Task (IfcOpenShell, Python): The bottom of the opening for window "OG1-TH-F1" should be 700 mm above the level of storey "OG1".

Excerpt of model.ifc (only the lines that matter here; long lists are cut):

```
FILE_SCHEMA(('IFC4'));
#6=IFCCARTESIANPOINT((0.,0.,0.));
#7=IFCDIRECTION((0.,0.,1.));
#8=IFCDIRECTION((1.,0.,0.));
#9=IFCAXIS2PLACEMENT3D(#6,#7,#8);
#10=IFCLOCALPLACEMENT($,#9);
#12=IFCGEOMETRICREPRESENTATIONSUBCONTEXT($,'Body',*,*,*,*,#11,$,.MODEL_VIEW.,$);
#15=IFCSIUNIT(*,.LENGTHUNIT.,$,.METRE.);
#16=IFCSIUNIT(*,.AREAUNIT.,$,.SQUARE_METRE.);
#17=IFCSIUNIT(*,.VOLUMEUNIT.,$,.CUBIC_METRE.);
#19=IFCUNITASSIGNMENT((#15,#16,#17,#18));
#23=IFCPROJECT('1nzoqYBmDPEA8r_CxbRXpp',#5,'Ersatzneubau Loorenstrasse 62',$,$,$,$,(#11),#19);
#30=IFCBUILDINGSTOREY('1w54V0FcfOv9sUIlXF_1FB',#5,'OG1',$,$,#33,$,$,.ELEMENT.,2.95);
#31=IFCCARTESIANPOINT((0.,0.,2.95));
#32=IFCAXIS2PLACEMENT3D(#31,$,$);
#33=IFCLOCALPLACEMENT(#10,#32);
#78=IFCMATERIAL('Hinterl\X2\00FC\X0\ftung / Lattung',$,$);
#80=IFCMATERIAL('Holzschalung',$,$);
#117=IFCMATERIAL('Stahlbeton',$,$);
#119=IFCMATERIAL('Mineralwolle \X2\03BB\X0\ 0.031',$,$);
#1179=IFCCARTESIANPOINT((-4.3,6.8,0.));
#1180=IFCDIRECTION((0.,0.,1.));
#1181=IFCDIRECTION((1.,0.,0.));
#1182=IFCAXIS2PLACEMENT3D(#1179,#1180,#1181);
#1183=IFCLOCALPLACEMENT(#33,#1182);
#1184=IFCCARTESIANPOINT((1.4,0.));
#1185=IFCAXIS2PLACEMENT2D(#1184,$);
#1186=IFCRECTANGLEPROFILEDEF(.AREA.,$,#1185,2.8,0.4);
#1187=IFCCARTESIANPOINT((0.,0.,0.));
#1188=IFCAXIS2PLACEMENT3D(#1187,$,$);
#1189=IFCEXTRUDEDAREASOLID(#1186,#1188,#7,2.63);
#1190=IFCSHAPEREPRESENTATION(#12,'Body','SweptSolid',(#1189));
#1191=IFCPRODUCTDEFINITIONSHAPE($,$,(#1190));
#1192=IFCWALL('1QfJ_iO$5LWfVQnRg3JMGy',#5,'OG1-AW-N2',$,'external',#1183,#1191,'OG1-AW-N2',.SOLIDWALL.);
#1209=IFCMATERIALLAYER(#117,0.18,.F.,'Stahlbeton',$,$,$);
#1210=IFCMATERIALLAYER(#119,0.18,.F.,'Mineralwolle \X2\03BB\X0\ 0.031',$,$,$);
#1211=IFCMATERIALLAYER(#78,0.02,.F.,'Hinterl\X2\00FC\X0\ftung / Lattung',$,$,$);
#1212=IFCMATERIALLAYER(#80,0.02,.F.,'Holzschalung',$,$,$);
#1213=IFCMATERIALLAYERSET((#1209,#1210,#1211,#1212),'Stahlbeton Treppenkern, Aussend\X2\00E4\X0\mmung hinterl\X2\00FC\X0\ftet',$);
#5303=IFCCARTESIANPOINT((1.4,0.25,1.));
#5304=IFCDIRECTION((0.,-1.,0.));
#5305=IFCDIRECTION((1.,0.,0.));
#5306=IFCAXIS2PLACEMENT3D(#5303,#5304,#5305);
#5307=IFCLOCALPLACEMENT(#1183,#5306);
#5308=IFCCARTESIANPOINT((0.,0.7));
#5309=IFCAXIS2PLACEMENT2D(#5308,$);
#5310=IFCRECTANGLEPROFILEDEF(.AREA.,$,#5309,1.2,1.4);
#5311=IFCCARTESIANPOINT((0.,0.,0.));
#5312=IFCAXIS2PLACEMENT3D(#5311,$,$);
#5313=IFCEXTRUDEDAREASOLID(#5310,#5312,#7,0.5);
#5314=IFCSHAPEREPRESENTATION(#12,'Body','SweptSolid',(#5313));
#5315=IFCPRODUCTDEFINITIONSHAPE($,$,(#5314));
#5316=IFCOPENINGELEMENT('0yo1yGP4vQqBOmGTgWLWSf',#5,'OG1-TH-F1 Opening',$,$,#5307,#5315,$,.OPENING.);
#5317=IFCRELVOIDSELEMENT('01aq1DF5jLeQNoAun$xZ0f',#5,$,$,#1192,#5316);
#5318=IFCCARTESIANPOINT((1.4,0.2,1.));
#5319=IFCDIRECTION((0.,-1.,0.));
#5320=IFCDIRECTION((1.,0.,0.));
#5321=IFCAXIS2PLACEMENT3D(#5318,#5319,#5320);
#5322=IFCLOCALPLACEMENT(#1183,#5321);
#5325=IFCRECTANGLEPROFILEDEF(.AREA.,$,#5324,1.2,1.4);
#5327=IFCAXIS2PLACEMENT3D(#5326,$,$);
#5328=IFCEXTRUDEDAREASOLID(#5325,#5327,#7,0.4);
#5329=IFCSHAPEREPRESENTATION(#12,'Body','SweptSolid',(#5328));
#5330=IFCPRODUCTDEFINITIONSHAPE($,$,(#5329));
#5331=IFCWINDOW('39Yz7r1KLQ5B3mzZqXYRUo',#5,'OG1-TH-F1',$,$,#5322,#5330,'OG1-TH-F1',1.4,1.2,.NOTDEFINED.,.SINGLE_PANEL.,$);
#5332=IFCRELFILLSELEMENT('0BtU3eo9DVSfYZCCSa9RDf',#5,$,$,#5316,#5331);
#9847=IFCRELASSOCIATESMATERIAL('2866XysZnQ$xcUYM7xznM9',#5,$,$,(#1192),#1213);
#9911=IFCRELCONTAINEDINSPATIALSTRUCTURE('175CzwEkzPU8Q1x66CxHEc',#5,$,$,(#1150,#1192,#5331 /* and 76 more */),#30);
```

```python
import numpy as np
import ifcopenshell
import ifcopenshell.api.geometry
import ifcopenshell.geom
import ifcopenshell.util.element
import ifcopenshell.util.placement
import ifcopenshell.util.shape
import ifcopenshell.util.unit

model = ifcopenshell.open("model.ifc")
unit_scale = ifcopenshell.util.unit.calculate_unit_scale(model)

window = model.by_id(5331)
opening = window.FillsVoids[0].RelatingOpeningElement
storey = ifcopenshell.util.element.get_container(window, ifc_class="IfcBuildingStorey")
level = ifcopenshell.util.placement.get_local_placement(storey.ObjectPlacement)[2, 3]

# The opening's origin need not be at the sill, so measure its lowest point.
shape = ifcopenshell.geom.create_shape(ifcopenshell.geom.settings(), opening)
bottom = ifcopenshell.util.shape.get_shape_bottom_elevation(shape, shape.geometry) / unit_scale
dz = level + 0.7 / unit_scale - bottom

shift = np.array([0.0, 0.0, dz])
# The window is not placed relative to its opening, so move both.
for product in (opening, window):
    matrix = ifcopenshell.util.placement.get_local_placement(product.ObjectPlacement)
    matrix[:3, 3] += shift
    ifcopenshell.api.geometry.edit_object_placement(model, product=product, matrix=matrix, is_si=False)

print(f"moved by {dz * unit_scale:+.3f} m")

model.write("model_updated.ifc")
```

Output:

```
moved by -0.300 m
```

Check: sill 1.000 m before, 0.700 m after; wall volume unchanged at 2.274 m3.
